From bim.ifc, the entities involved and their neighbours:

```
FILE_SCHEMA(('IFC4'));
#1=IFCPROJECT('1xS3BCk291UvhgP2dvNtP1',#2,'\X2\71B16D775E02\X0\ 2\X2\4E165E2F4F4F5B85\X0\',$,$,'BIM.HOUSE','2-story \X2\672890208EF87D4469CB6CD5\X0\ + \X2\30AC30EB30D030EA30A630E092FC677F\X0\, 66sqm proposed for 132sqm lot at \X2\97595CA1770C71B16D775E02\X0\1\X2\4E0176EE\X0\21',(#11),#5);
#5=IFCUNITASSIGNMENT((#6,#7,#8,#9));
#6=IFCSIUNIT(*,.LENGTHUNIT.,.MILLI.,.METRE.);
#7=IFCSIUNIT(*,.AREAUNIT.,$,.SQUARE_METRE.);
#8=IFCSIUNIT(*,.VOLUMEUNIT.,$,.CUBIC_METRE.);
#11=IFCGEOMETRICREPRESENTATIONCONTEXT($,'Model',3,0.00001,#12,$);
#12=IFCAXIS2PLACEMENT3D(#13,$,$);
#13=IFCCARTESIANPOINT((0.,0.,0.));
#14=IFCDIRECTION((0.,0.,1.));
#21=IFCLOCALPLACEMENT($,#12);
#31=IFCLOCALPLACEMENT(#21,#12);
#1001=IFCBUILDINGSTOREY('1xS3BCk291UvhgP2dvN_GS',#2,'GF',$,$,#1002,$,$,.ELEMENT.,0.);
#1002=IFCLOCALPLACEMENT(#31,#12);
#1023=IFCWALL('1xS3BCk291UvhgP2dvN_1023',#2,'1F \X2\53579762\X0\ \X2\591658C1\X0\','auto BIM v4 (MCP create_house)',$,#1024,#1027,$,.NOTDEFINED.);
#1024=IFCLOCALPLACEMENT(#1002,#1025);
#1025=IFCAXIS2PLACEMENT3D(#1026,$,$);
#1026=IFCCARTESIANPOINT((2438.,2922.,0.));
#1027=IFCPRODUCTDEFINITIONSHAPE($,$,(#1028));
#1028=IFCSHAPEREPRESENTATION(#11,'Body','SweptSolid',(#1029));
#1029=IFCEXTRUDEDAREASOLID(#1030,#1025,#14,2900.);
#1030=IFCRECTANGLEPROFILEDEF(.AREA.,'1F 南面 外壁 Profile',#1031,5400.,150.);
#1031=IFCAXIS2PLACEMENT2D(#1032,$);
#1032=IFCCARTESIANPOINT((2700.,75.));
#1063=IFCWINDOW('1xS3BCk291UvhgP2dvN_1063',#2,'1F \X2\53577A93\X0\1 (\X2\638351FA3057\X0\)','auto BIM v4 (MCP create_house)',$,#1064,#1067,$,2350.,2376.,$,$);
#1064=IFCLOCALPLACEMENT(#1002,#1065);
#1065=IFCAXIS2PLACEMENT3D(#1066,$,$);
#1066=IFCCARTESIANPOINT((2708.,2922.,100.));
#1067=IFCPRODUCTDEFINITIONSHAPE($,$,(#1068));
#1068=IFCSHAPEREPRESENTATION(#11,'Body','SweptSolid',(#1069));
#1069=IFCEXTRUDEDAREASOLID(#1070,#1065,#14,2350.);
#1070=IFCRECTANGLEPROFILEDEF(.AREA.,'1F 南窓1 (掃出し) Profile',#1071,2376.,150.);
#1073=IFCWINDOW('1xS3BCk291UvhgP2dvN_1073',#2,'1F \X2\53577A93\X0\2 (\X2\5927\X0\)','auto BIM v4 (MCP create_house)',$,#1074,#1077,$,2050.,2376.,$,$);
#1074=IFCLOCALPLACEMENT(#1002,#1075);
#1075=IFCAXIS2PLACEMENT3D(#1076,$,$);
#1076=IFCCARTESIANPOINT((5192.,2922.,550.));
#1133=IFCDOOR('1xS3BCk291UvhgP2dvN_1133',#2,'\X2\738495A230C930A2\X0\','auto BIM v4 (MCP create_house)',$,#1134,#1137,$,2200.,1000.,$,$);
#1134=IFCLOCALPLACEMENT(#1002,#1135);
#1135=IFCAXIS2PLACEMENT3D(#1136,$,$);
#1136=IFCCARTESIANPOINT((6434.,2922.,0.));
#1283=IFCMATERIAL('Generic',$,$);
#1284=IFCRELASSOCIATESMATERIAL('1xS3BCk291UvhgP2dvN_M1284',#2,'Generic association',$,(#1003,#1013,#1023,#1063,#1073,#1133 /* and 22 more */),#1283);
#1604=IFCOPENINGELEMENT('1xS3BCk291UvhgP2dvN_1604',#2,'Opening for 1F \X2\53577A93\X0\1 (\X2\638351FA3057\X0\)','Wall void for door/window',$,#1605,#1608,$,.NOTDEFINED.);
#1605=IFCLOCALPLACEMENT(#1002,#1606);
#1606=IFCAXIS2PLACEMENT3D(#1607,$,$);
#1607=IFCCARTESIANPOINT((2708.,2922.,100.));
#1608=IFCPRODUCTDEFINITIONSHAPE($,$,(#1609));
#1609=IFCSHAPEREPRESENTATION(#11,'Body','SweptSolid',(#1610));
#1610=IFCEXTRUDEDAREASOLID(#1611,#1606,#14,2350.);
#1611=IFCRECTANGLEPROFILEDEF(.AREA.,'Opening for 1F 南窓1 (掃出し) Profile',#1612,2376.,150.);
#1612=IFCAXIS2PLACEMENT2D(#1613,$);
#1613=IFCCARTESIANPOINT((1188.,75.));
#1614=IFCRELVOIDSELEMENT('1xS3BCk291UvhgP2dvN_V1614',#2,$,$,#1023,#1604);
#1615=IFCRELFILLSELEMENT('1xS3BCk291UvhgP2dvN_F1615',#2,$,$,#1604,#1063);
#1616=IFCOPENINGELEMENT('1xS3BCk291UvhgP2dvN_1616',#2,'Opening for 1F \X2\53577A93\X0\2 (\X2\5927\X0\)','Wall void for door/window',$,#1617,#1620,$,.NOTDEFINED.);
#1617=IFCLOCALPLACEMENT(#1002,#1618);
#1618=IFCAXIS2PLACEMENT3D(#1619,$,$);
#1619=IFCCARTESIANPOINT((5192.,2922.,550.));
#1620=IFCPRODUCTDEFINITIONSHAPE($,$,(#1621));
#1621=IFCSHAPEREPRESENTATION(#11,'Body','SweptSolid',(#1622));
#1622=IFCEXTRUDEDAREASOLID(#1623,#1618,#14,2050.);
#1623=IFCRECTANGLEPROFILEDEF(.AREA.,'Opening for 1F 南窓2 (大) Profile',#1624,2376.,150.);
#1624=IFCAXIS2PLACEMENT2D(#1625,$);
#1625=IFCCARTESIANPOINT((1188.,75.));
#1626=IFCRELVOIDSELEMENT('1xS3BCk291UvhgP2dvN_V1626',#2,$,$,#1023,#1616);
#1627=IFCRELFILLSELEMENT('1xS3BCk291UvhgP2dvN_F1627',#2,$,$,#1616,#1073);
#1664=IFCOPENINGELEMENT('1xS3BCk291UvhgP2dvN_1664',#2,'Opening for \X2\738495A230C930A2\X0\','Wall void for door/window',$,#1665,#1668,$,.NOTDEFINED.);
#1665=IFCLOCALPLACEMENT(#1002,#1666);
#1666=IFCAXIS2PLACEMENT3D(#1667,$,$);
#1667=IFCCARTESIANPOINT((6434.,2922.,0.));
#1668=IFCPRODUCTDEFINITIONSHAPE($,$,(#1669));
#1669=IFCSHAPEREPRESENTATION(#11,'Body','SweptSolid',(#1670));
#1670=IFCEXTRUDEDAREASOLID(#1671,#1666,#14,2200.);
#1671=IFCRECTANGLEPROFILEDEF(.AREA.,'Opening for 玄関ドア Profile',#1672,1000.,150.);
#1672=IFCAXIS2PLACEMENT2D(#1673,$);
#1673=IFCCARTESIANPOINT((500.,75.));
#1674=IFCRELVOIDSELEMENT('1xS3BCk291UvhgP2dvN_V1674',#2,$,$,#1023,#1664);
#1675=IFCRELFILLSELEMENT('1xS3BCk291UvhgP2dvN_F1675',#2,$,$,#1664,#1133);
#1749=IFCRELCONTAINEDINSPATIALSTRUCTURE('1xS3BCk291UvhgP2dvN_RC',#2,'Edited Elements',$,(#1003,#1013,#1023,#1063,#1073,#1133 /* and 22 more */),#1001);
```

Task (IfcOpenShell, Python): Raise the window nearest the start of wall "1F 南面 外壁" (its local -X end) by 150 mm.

```python
import numpy as np
import ifcopenshell
import ifcopenshell.api.geometry
import ifcopenshell.util.placement
import ifcopenshell.util.unit

model = ifcopenshell.open("bim.ifc")
unit_scale = ifcopenshell.util.unit.calculate_unit_scale(model)

window = model.by_id(1063)
opening = window.FillsVoids[0].RelatingOpeningElement
dz = 0.15 / unit_scale

shift = np.array([0.0, 0.0, dz])
# The window is not placed relative to its opening, so move both.
for product in (opening, window):
    matrix = ifcopenshell.util.placement.get_local_placement(product.ObjectPlacement)
    matrix[:3, 3] += shift
    ifcopenshell.api.geometry.edit_object_placement(model, product=product, matrix=matrix, is_si=False)

print(f"moved by {dz * unit_scale:+.3f} m")

model.write("bim_updated.ifc")
```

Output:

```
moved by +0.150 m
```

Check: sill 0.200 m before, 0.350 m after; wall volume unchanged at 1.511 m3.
